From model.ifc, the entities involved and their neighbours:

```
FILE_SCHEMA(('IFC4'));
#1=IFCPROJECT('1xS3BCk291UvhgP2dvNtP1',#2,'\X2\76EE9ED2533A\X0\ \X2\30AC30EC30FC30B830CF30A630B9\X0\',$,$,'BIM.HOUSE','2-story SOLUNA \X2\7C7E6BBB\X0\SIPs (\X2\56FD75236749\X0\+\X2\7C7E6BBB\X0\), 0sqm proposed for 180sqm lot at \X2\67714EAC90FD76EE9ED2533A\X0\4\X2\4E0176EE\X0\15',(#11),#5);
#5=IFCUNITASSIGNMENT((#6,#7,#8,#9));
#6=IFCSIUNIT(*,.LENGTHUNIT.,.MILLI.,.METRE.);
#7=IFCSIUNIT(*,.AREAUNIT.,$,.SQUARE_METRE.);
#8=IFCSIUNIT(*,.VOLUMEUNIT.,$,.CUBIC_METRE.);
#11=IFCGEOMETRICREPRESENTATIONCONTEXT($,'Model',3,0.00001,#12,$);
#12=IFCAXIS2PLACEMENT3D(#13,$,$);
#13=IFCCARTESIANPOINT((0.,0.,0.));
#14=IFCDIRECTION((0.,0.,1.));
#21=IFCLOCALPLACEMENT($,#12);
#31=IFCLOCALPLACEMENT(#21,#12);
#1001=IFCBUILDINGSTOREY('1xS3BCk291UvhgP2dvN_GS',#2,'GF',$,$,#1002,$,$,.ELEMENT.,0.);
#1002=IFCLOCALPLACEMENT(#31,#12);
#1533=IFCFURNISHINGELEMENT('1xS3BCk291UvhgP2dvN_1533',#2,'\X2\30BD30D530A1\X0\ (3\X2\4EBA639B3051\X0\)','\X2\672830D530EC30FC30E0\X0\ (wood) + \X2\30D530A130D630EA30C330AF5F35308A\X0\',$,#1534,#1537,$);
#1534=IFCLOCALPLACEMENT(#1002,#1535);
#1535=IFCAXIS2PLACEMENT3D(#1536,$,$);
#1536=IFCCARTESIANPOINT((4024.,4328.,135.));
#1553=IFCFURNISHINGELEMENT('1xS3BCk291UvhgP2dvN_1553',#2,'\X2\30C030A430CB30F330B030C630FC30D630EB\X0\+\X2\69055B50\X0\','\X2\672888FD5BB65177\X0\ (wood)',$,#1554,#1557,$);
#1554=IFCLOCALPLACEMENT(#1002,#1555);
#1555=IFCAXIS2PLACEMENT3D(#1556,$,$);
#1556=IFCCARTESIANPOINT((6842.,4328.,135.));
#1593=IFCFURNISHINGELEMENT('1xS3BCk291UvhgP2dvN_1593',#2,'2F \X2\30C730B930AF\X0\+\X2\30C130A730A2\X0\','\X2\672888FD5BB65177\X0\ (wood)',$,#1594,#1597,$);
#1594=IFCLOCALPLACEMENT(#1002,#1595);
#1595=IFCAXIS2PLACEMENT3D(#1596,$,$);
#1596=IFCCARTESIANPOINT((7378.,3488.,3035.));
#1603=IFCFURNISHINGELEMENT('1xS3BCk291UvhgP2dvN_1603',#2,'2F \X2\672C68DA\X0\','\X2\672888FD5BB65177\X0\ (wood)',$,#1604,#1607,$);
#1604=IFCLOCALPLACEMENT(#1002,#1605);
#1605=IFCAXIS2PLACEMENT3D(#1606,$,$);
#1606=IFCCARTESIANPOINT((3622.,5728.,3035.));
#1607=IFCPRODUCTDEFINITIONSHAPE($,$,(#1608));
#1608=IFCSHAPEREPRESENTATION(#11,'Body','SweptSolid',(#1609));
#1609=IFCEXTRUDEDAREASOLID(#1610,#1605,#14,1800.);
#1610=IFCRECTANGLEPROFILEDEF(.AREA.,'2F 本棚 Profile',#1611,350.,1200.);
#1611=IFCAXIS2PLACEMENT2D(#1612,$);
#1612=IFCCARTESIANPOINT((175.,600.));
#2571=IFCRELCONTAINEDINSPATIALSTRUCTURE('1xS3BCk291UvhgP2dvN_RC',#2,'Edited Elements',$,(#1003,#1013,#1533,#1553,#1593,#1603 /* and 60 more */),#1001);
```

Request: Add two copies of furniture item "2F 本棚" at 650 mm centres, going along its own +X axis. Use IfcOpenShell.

```python
import ifcopenshell
import ifcopenshell.api.geometry
import ifcopenshell.api.root
import ifcopenshell.util.element
import ifcopenshell.util.placement
import ifcopenshell.util.unit

model = ifcopenshell.open("model.ifc")
unit_scale = ifcopenshell.util.unit.calculate_unit_scale(model)


def reuse_history(source, copy):
    """copy_class also copies each property set's owner history, people and application; keep the originals."""
    for rel in copy.IsDefinedBy:
        if rel.is_a("IfcRelDefinesByProperties") and (history := rel.RelatingPropertyDefinition.OwnerHistory):
            rel.RelatingPropertyDefinition.OwnerHistory = source.OwnerHistory
            ifcopenshell.util.element.remove_deep2(model, history)


source = model.by_guid("1xS3BCk291UvhgP2dvN_1603")
base = ifcopenshell.util.placement.get_local_placement(source.ObjectPlacement)
step = base[:3, 0] * 0.65 / unit_scale

for i in range(1, 3):
    copy = ifcopenshell.api.root.copy_class(model, product=source)
    copy.Representation = ifcopenshell.util.element.copy_deep(
        model, source.Representation, exclude=["IfcGeometricRepresentationContext", "IfcRepresentationMap"]
    )
    reuse_history(source, copy)
    matrix = base.copy()
    matrix[:3, 3] += i * step
    print("added at", matrix[:3, 3].round(3) + 0.0)
    ifcopenshell.api.geometry.edit_object_placement(model, product=copy, matrix=matrix, is_si=False)

model.write("model_edited.ifc")
```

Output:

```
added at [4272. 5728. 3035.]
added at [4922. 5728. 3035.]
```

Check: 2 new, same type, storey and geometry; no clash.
